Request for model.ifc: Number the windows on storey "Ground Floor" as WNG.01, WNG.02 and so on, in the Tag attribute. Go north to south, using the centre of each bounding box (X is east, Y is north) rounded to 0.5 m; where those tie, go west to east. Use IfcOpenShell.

First a look at what the model holds.

```python
import ifcopenshell
import ifcopenshell.util.element
import ifcopenshell.util.placement

model = ifcopenshell.open("model.ifc")
print(model.schema)
storey = next(s for s in model.by_type("IfcBuildingStorey") if s.Name == "Ground Floor")
windows = [e for e in ifcopenshell.util.element.get_decomposition(storey) if e.is_a("IfcWindow")]
for e in sorted(windows, key=lambda e: e.id()):
    origin = ifcopenshell.util.placement.get_local_placement(e.ObjectPlacement)[:3, 3]
    print(e.id(), e.Tag, e.Name, origin.round(2) + 0.0, sep=" | ")
```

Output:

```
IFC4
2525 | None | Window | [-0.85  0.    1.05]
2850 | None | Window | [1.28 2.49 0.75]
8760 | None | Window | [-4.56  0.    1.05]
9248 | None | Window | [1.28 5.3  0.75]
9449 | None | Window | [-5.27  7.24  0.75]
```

```python
import ifcopenshell
import ifcopenshell.geom
import ifcopenshell.util.element
import ifcopenshell.util.shape

model = ifcopenshell.open("model.ifc")
settings = ifcopenshell.geom.settings()
settings.set("use-world-coords", True)


def centre(element):
    shape = ifcopenshell.geom.create_shape(settings, element)
    return ifcopenshell.util.shape.get_bbox_centroid(shape.geometry)


storey = next(s for s in model.by_type("IfcBuildingStorey") if s.Name == "Ground Floor")
windows = [e for e in ifcopenshell.util.element.get_decomposition(storey) if e.is_a("IfcWindow")]

# Insertion points can sit at a corner or the storey origin, so sort by the geometry (in metres).
centres = {e: centre(e) for e in windows}
windows.sort(key=lambda e: (-round(centres[e][1] / 0.5), centres[e][0]))

for i, e in enumerate(windows, start=1):
    number = f"WNG.{i:02d}"
    e.Tag = number
    print(e.id(), number)

model.write("model_edited.ifc")
```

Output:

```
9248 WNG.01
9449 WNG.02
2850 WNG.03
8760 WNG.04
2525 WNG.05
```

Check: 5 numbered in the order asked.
